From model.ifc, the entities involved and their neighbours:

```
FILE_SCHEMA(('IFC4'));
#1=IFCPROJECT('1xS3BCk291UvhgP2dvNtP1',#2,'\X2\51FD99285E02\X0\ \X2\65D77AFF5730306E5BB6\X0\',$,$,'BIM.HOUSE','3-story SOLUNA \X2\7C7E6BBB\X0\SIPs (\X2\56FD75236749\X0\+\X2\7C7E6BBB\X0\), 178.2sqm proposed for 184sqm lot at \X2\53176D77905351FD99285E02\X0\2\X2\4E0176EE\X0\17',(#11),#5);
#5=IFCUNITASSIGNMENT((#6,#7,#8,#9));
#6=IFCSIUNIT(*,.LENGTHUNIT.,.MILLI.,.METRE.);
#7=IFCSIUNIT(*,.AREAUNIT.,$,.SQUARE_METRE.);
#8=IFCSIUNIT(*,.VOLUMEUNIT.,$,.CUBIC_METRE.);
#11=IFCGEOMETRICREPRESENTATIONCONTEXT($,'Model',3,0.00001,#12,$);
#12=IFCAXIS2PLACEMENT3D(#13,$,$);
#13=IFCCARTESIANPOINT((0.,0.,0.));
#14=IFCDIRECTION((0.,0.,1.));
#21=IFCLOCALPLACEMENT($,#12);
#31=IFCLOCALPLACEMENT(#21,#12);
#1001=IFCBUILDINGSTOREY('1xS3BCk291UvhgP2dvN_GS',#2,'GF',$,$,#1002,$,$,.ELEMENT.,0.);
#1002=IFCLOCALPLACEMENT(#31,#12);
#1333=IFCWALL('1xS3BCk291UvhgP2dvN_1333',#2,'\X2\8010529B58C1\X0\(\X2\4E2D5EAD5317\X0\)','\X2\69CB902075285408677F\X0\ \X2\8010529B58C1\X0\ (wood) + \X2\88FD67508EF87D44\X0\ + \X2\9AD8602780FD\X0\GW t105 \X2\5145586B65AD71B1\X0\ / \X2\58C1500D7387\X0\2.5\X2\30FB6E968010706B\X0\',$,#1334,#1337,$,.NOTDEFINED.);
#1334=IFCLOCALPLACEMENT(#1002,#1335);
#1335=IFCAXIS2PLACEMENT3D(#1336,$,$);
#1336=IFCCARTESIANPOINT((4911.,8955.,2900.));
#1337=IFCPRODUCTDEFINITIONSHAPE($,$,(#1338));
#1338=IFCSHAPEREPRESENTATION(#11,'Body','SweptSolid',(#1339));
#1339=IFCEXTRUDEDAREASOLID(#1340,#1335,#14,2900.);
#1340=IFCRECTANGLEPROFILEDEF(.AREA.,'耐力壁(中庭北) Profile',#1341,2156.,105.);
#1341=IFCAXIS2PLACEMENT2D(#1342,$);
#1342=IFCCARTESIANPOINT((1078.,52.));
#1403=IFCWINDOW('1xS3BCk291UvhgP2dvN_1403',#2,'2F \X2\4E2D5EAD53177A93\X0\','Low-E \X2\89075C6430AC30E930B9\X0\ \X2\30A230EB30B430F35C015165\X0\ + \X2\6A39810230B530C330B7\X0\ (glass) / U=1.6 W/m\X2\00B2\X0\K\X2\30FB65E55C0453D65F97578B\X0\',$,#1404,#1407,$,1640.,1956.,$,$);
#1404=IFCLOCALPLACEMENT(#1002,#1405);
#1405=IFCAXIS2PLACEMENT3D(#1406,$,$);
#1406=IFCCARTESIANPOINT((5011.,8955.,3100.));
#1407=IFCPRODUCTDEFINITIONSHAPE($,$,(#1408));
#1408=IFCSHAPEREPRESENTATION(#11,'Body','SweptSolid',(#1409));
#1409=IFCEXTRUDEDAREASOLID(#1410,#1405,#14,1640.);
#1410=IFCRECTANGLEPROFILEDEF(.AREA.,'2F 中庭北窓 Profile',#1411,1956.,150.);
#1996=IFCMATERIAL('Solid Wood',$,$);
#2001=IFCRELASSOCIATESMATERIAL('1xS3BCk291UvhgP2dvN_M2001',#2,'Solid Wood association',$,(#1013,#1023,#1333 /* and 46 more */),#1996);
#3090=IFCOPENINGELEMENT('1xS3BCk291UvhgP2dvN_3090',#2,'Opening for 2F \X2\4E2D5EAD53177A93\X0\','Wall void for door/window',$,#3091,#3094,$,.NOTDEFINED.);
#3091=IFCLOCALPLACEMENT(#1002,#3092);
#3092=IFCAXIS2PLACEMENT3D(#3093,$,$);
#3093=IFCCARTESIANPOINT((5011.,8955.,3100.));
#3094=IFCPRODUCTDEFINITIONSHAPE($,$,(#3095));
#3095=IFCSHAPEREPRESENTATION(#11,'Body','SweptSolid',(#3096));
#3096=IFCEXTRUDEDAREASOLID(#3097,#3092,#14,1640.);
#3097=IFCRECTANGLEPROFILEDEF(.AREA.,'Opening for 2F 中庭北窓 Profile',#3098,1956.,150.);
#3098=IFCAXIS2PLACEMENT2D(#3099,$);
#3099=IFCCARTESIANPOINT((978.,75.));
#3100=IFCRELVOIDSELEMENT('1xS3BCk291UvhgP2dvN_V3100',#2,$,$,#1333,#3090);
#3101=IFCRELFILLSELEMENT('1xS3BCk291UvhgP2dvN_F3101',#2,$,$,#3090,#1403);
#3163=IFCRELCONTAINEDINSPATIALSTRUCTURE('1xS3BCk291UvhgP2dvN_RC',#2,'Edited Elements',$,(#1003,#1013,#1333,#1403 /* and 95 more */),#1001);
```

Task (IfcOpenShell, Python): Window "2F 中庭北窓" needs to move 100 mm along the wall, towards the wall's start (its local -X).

```python
import ifcopenshell
import ifcopenshell.api.geometry
import ifcopenshell.util.placement
import ifcopenshell.util.unit

model = ifcopenshell.open("model.ifc")
unit_scale = ifcopenshell.util.unit.calculate_unit_scale(model)

window = model.by_guid("1xS3BCk291UvhgP2dvN_1403")
opening = window.FillsVoids[0].RelatingOpeningElement
wall = opening.VoidsElements[0].RelatingBuildingElement

wall_matrix = ifcopenshell.util.placement.get_local_placement(wall.ObjectPlacement)
shift = wall_matrix[:3, 0] * -0.1 / unit_scale
before = ifcopenshell.util.placement.get_local_placement(window.ObjectPlacement)[:3, 3].copy()

# The window is not placed relative to its opening, so move both.
for product in (opening, window):
    matrix = ifcopenshell.util.placement.get_local_placement(product.ObjectPlacement)
    matrix[:3, 3] += shift
    ifcopenshell.api.geometry.edit_object_placement(model, product=product, matrix=matrix, is_si=False)

after = ifcopenshell.util.placement.get_local_placement(window.ObjectPlacement)[:3, 3]
print("window moved by", (after - before).round(3) + 0.0)

model.write("model_updated.ifc")
```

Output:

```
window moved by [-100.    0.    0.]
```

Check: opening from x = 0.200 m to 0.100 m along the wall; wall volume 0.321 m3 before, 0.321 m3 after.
